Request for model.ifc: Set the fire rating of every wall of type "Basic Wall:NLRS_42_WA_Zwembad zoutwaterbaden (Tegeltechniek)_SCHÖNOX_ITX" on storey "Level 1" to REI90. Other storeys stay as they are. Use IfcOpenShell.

First a look at what the model holds.

```python
import ifcopenshell
import ifcopenshell.util.element

model = ifcopenshell.open("model.ifc")
print(model.schema)
storey = next(s for s in model.by_type("IfcBuildingStorey") if s.Name == "Level 1")
walls = [e for e in ifcopenshell.util.element.get_decomposition(storey) if e.is_a("IfcWall")]
seen = {}
for e in walls:
    element_type = ifcopenshell.util.element.get_type(e)
    key = (element_type.Name if element_type != e and element_type else None, ifcopenshell.util.element.get_pset(e, "Pset_WallCommon", "FireRating"))
    seen[key] = seen.get(key, 0) + 1
for (name, value), count in sorted(seen.items(), key=str):
    print(count, "x", name, "|", value)
```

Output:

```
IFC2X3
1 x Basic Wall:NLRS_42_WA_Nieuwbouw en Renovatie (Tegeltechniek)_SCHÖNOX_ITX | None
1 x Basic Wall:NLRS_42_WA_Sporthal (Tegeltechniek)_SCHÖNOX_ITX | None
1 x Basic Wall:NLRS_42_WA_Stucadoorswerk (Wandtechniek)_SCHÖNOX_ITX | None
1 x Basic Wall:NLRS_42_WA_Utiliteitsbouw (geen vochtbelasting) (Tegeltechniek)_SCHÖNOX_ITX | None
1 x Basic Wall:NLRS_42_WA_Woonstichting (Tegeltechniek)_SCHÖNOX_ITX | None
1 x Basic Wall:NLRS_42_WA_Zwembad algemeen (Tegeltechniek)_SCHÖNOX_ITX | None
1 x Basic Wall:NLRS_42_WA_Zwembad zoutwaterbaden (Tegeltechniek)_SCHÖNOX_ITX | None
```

```python
import ifcopenshell
import ifcopenshell.api.pset
import ifcopenshell.util.element

model = ifcopenshell.open("model.ifc")

storey = next(s for s in model.by_type("IfcBuildingStorey") if s.Name == "Level 1")
walls = [e for e in ifcopenshell.util.element.get_decomposition(storey) if e.is_a("IfcWall")]

count = 0
for e in walls:
    element_type = ifcopenshell.util.element.get_type(e)
    if element_type in (None, e) or element_type.Name != "Basic Wall:NLRS_42_WA_Zwembad zoutwaterbaden (Tegeltechniek)_SCHÖNOX_ITX":
        continue
    # add_pset returns the element's existing set when there is one.
    pset = ifcopenshell.api.pset.add_pset(model, product=e, name="Pset_WallCommon")
    ifcopenshell.api.pset.edit_pset(model, pset=pset, properties={"FireRating": "REI90"})
    count += 1

print(count, "walls updated")

model.write("model_updated.ifc")
```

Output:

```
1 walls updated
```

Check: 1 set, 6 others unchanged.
